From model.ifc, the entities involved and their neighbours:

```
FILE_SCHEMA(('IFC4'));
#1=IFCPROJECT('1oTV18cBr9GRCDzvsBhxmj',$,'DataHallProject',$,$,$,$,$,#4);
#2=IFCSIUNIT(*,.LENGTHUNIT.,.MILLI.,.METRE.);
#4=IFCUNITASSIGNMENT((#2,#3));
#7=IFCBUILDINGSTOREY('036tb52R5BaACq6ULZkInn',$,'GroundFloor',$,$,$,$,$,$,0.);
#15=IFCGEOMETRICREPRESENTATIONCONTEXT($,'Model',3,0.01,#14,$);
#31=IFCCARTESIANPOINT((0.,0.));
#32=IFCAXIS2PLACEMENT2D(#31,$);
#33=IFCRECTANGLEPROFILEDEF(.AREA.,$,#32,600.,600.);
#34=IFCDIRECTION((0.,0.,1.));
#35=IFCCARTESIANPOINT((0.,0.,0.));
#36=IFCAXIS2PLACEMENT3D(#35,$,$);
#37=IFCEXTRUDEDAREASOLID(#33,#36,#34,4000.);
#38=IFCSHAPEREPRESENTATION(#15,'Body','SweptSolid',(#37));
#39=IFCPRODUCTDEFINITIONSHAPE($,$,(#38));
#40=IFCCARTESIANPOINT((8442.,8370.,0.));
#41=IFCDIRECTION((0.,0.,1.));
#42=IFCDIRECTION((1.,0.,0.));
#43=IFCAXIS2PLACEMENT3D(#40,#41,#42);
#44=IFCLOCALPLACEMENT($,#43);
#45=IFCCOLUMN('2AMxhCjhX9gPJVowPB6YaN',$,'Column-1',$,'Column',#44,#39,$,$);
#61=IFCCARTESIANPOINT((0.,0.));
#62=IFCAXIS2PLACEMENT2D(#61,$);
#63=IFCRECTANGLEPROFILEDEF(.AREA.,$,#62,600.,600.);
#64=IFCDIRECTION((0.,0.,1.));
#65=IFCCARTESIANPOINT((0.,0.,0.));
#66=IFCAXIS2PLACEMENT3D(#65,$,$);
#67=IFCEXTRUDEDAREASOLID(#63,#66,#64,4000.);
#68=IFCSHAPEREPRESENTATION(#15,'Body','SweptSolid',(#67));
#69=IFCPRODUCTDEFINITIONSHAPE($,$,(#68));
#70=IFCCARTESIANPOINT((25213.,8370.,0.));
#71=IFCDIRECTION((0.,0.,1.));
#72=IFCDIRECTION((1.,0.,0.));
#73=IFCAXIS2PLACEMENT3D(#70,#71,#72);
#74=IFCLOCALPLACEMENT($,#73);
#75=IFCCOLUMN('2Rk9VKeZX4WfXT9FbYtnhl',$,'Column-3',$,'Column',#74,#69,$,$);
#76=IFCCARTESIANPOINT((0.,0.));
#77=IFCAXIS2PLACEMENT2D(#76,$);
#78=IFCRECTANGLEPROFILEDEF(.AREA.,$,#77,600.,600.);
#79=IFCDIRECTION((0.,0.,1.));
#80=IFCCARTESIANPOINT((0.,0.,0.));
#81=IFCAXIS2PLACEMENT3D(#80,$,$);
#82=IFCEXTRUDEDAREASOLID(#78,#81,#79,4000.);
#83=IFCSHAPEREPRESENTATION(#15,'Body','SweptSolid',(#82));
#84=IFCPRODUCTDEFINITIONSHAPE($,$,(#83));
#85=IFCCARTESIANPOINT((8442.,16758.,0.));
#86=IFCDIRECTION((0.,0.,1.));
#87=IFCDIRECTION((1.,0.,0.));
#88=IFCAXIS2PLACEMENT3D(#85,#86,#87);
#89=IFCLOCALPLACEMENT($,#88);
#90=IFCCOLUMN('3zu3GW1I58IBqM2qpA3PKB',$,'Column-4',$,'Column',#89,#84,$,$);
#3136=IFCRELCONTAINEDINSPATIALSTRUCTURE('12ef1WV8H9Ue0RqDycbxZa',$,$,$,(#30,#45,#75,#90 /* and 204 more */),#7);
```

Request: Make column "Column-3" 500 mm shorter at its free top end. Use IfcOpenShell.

```python
import ifcopenshell

model = ifcopenshell.open("model.ifc")

member = model.by_guid("2Rk9VKeZX4WfXT9FbYtnhl")
change = -500.0

# The extrusion runs towards the end named, so only its depth changes.
body = next(r for r in member.Representation.Representations if r.RepresentationIdentifier == "Body")
solid = body.Items[0]
old_length = solid.Depth
solid.Depth += change

print(f"length {old_length:g} -> {solid.Depth:g}")

model.write("model_rev.ifc")
```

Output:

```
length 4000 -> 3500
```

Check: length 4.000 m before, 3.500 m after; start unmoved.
